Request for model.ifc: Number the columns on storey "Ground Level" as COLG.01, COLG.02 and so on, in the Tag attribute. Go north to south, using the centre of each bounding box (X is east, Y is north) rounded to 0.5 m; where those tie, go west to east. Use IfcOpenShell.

First a look at what the model holds.

```python
import ifcopenshell
import ifcopenshell.util.element
import ifcopenshell.util.placement

model = ifcopenshell.open("model.ifc")
print(model.schema)
storey = next(s for s in model.by_type("IfcBuildingStorey") if s.Name == "Ground Level")
columns = [e for e in ifcopenshell.util.element.get_decomposition(storey) if e.is_a("IfcColumn")]
for e in sorted(columns, key=lambda e: e.id()):
    origin = ifcopenshell.util.placement.get_local_placement(e.ObjectPlacement)[:3, 3]
    print(e.id(), e.Tag, e.Name, origin.round(2) + 0.0, sep=" | ")
```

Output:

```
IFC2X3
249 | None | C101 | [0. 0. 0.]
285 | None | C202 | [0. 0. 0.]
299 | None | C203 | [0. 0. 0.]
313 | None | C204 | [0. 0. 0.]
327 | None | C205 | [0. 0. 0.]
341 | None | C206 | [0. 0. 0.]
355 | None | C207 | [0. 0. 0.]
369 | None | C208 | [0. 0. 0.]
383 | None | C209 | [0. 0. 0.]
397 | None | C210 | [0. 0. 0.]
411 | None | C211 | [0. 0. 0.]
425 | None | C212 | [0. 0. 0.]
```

```python
import ifcopenshell
import ifcopenshell.geom
import ifcopenshell.util.element
import ifcopenshell.util.shape

model = ifcopenshell.open("model.ifc")
settings = ifcopenshell.geom.settings()
settings.set("use-world-coords", True)


def centre(element):
    shape = ifcopenshell.geom.create_shape(settings, element)
    return ifcopenshell.util.shape.get_bbox_centroid(shape.geometry)


storey = next(s for s in model.by_type("IfcBuildingStorey") if s.Name == "Ground Level")
columns = [e for e in ifcopenshell.util.element.get_decomposition(storey) if e.is_a("IfcColumn")]

# Insertion points can sit at a corner or the storey origin, so sort by the geometry (in metres).
centres = {e: centre(e) for e in columns}
columns.sort(key=lambda e: (-round(centres[e][1] / 0.5), centres[e][0]))

for i, e in enumerate(columns, start=1):
    number = f"COLG.{i:02d}"
    e.Tag = number
    print(e.id(), number)

model.write("model_rev.ifc")
```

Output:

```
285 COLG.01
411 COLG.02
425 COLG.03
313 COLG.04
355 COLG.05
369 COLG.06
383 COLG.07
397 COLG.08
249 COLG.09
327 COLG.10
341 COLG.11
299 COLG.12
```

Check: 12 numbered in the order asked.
